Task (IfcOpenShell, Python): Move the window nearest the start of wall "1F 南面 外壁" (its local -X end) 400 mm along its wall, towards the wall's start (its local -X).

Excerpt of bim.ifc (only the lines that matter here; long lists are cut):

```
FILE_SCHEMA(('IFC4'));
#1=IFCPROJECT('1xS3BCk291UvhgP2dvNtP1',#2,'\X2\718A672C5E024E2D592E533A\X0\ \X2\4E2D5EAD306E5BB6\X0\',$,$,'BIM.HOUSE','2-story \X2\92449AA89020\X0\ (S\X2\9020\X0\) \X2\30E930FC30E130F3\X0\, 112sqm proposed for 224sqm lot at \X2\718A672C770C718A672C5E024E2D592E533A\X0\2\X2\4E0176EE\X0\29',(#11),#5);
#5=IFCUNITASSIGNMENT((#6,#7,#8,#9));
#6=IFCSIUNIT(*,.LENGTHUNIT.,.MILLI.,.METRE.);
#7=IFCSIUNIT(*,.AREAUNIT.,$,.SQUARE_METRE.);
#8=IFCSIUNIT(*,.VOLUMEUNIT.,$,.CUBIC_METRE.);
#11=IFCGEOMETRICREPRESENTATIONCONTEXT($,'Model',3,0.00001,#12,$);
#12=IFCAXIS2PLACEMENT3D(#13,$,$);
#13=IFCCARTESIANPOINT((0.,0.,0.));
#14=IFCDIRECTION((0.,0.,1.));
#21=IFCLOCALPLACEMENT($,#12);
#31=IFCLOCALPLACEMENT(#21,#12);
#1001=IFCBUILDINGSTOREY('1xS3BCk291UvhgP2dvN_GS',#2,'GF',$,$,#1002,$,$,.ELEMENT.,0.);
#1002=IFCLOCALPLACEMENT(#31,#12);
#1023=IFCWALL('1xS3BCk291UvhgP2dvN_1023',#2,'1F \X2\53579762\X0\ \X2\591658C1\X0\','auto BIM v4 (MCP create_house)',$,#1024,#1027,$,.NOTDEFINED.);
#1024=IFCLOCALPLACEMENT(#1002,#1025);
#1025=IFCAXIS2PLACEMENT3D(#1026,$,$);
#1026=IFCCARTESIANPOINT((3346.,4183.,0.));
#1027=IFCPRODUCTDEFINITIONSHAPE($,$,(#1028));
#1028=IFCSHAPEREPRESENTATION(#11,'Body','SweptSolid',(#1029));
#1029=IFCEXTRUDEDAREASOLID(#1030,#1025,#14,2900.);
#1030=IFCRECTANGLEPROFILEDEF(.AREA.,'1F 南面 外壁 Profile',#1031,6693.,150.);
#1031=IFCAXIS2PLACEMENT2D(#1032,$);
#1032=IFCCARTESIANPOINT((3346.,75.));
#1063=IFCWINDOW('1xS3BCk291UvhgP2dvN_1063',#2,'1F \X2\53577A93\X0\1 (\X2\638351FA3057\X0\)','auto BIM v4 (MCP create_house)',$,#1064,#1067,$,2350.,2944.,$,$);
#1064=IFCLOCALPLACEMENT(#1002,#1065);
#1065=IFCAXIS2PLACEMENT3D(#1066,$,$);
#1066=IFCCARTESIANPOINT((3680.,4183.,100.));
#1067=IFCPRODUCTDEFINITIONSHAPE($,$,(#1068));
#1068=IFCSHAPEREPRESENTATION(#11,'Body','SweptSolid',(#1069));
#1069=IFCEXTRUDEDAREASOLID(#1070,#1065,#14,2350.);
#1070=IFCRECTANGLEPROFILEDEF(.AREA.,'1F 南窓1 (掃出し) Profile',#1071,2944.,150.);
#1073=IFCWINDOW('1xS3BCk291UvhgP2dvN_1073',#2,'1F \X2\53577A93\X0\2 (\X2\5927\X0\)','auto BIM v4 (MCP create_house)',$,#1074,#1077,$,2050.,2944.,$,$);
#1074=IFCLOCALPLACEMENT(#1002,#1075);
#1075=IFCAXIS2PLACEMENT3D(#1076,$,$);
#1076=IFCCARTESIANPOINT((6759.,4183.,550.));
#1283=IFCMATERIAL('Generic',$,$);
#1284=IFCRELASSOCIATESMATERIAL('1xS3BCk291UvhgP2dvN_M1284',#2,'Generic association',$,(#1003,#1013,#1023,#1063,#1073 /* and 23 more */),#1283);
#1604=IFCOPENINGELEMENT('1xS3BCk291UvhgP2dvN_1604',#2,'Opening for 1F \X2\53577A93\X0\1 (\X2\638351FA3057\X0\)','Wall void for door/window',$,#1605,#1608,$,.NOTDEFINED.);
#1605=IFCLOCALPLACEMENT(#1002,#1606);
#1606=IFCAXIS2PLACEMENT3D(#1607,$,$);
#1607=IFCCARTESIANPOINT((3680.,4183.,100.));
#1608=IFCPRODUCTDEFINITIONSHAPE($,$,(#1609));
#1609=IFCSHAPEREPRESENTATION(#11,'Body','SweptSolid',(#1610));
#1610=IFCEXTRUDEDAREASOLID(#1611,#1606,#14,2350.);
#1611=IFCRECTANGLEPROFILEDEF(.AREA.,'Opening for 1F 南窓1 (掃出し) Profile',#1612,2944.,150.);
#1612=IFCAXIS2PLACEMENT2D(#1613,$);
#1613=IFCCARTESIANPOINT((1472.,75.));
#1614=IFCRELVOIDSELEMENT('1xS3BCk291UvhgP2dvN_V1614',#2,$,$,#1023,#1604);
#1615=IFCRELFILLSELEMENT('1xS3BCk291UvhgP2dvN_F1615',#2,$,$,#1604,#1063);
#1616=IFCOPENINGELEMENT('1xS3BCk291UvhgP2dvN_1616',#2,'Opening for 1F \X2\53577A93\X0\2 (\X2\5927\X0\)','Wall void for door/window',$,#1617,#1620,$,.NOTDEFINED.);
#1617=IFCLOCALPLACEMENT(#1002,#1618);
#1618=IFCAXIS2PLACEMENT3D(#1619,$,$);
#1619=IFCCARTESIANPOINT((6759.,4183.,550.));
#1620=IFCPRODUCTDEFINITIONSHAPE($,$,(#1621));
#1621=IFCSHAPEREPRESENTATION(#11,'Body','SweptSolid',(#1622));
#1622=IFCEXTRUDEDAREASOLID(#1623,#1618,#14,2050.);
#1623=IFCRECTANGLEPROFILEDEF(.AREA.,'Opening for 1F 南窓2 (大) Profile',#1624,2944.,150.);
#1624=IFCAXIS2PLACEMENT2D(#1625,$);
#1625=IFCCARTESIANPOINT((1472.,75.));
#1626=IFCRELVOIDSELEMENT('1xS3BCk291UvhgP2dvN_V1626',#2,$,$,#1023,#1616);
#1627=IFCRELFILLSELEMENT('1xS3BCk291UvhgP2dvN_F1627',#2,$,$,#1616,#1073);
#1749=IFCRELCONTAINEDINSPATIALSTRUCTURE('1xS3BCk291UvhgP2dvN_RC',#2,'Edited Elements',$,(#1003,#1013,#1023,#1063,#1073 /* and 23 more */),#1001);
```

```python
import ifcopenshell
import ifcopenshell.api.geometry
import ifcopenshell.util.placement
import ifcopenshell.util.unit

model = ifcopenshell.open("bim.ifc")
unit_scale = ifcopenshell.util.unit.calculate_unit_scale(model)

window = model.by_guid("1xS3BCk291UvhgP2dvN_1063")
opening = window.FillsVoids[0].RelatingOpeningElement
wall = opening.VoidsElements[0].RelatingBuildingElement

wall_matrix = ifcopenshell.util.placement.get_local_placement(wall.ObjectPlacement)
shift = wall_matrix[:3, 0] * -0.4 / unit_scale
before = ifcopenshell.util.placement.get_local_placement(window.ObjectPlacement)[:3, 3].copy()

# The window is not placed relative to its opening, so move both.
for product in (opening, window):
    matrix = ifcopenshell.util.placement.get_local_placement(product.ObjectPlacement)
    matrix[:3, 3] += shift
    ifcopenshell.api.geometry.edit_object_placement(model, product=product, matrix=matrix, is_si=False)

after = ifcopenshell.util.placement.get_local_placement(window.ObjectPlacement)[:3, 3]
print("window moved by", (after - before).round(3) + 0.0)

model.write("bim_updated.ifc")
```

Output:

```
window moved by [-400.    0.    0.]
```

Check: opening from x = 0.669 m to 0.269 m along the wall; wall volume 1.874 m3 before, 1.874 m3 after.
